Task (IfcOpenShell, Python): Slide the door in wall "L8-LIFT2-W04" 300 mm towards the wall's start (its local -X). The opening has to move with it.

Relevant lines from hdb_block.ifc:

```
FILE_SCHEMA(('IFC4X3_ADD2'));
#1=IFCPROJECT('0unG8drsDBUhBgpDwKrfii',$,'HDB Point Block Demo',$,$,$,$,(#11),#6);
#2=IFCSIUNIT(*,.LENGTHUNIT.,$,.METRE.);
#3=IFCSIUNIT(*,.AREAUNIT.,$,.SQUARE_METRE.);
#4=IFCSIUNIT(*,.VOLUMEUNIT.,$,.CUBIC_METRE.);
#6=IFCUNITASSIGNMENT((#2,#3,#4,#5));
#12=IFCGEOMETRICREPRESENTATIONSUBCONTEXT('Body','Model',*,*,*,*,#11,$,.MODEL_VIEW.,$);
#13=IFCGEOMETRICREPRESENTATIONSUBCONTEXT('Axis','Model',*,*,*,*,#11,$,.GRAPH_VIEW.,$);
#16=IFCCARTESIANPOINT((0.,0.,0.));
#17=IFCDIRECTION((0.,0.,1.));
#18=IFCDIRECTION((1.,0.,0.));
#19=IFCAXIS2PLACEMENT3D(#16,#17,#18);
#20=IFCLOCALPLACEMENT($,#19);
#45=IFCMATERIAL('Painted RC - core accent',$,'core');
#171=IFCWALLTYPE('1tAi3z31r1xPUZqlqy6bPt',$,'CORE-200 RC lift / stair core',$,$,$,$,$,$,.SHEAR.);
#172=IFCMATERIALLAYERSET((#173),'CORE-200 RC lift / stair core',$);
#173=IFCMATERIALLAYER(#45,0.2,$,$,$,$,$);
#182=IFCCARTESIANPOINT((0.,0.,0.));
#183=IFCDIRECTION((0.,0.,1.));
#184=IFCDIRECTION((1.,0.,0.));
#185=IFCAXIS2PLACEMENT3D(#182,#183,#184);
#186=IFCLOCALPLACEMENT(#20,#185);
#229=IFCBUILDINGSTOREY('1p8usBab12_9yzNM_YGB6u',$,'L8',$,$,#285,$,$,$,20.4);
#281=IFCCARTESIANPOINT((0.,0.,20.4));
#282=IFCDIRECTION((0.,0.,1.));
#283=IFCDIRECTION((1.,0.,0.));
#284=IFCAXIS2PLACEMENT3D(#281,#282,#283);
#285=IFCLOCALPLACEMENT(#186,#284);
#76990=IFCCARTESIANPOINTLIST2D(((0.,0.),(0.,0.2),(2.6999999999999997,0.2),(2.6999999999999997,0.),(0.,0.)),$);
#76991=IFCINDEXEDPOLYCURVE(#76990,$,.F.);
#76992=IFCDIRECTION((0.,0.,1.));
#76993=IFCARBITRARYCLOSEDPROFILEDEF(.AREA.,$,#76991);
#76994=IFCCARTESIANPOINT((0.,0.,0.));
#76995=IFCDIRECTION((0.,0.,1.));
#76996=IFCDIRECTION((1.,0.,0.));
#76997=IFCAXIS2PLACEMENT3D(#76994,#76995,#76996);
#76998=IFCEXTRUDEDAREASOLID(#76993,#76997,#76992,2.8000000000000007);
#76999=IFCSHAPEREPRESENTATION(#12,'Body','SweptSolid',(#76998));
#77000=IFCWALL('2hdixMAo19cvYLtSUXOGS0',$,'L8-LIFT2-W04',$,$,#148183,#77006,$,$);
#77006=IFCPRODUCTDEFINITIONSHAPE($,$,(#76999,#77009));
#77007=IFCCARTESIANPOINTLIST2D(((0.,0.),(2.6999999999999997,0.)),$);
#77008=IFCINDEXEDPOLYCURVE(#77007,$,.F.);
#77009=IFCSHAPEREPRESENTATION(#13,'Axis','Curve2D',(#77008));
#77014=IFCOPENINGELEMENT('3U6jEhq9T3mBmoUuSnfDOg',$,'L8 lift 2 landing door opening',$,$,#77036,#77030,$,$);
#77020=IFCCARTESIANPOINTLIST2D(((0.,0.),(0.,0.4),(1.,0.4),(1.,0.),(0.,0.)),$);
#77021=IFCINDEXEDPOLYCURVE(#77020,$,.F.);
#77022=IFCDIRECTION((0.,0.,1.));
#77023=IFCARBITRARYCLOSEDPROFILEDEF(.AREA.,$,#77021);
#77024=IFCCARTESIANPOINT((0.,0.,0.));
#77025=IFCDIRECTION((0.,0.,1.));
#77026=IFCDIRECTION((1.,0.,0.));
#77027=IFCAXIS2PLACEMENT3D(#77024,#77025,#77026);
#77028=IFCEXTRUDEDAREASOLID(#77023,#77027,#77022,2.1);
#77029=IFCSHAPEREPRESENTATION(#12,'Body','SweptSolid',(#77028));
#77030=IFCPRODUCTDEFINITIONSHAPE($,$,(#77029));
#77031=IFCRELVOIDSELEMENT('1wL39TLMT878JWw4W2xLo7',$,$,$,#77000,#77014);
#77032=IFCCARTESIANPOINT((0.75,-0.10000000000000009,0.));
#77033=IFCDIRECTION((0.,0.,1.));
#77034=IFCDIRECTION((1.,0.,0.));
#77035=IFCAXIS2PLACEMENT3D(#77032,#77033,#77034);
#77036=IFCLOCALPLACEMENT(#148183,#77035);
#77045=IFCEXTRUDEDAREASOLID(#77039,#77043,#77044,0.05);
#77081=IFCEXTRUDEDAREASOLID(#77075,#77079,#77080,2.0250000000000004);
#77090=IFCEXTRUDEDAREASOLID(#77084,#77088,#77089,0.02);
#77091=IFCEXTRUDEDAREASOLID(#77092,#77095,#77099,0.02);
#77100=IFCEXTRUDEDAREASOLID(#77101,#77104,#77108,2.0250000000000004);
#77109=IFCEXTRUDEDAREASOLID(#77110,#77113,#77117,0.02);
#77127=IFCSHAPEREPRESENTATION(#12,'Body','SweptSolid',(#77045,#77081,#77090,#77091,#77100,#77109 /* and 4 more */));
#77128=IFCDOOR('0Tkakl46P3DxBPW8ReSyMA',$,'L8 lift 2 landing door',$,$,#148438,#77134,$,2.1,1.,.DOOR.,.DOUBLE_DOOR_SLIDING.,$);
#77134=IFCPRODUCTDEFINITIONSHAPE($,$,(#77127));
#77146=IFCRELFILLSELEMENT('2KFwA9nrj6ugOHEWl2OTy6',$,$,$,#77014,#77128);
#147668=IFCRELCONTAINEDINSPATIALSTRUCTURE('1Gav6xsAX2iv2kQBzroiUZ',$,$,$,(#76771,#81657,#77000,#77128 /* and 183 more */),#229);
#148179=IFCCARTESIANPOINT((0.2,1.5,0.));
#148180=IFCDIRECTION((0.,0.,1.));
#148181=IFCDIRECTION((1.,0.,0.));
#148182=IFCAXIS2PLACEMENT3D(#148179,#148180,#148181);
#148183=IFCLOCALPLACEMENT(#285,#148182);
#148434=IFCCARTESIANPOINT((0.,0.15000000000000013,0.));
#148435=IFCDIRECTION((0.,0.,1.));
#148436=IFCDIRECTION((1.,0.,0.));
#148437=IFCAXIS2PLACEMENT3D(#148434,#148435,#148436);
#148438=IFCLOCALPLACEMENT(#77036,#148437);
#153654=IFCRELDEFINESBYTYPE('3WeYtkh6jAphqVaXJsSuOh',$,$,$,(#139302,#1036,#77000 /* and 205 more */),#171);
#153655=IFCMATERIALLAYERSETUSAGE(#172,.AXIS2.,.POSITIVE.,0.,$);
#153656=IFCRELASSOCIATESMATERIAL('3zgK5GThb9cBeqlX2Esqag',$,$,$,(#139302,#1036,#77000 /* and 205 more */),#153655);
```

```python
import ifcopenshell
import ifcopenshell.api.geometry
import ifcopenshell.util.placement

model = ifcopenshell.open("hdb_block.ifc")

door = model.by_id(77128)
opening = door.FillsVoids[0].RelatingOpeningElement
wall = opening.VoidsElements[0].RelatingBuildingElement

wall_matrix = ifcopenshell.util.placement.get_local_placement(wall.ObjectPlacement)
shift = wall_matrix[:3, 0] * -0.3
before = ifcopenshell.util.placement.get_local_placement(door.ObjectPlacement)[:3, 3].copy()

# The door is placed relative to its opening, so it follows when the opening moves.
matrix = ifcopenshell.util.placement.get_local_placement(opening.ObjectPlacement)
matrix[:3, 3] += shift
ifcopenshell.api.geometry.edit_object_placement(
    model, product=opening, matrix=matrix, is_si=False, should_transform_children=True
)

after = ifcopenshell.util.placement.get_local_placement(door.ObjectPlacement)[:3, 3]
print("door moved by", (after - before).round(3) + 0.0)

model.write("hdb_block_edited.ifc")
```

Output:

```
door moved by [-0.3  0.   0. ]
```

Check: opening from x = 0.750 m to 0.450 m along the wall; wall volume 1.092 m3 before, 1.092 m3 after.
